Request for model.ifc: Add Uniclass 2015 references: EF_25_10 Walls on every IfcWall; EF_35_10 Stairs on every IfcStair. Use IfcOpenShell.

First a look at what the model holds.

```python
import ifcopenshell

model = ifcopenshell.open("model.ifc")
print(model.schema)
print("classifications:", [c.Name for c in model.by_type("IfcClassification")])
for ifc_class in ("IfcDoor", "IfcRoof", "IfcStair", "IfcWall", "IfcWindow"):
    print(ifc_class, len(model.by_type(ifc_class)))
```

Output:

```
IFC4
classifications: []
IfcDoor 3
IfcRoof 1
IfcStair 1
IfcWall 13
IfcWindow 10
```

```python
import ifcopenshell
import ifcopenshell.api.classification

model = ifcopenshell.open("model.ifc")

system = ifcopenshell.api.classification.add_classification(model, classification="Uniclass 2015")

codes = {
    "IfcWall": ("EF_25_10", "Walls"),
    "IfcStair": ("EF_35_10", "Stairs"),
}
for ifc_class, (code, name) in codes.items():
    products = model.by_type(ifc_class)
    ifcopenshell.api.classification.add_reference(
        model, products=products, classification=system, identification=code, name=name
    )
    print(code, len(products))

model.write("model_rev.ifc")
```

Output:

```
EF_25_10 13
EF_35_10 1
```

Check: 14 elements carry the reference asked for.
